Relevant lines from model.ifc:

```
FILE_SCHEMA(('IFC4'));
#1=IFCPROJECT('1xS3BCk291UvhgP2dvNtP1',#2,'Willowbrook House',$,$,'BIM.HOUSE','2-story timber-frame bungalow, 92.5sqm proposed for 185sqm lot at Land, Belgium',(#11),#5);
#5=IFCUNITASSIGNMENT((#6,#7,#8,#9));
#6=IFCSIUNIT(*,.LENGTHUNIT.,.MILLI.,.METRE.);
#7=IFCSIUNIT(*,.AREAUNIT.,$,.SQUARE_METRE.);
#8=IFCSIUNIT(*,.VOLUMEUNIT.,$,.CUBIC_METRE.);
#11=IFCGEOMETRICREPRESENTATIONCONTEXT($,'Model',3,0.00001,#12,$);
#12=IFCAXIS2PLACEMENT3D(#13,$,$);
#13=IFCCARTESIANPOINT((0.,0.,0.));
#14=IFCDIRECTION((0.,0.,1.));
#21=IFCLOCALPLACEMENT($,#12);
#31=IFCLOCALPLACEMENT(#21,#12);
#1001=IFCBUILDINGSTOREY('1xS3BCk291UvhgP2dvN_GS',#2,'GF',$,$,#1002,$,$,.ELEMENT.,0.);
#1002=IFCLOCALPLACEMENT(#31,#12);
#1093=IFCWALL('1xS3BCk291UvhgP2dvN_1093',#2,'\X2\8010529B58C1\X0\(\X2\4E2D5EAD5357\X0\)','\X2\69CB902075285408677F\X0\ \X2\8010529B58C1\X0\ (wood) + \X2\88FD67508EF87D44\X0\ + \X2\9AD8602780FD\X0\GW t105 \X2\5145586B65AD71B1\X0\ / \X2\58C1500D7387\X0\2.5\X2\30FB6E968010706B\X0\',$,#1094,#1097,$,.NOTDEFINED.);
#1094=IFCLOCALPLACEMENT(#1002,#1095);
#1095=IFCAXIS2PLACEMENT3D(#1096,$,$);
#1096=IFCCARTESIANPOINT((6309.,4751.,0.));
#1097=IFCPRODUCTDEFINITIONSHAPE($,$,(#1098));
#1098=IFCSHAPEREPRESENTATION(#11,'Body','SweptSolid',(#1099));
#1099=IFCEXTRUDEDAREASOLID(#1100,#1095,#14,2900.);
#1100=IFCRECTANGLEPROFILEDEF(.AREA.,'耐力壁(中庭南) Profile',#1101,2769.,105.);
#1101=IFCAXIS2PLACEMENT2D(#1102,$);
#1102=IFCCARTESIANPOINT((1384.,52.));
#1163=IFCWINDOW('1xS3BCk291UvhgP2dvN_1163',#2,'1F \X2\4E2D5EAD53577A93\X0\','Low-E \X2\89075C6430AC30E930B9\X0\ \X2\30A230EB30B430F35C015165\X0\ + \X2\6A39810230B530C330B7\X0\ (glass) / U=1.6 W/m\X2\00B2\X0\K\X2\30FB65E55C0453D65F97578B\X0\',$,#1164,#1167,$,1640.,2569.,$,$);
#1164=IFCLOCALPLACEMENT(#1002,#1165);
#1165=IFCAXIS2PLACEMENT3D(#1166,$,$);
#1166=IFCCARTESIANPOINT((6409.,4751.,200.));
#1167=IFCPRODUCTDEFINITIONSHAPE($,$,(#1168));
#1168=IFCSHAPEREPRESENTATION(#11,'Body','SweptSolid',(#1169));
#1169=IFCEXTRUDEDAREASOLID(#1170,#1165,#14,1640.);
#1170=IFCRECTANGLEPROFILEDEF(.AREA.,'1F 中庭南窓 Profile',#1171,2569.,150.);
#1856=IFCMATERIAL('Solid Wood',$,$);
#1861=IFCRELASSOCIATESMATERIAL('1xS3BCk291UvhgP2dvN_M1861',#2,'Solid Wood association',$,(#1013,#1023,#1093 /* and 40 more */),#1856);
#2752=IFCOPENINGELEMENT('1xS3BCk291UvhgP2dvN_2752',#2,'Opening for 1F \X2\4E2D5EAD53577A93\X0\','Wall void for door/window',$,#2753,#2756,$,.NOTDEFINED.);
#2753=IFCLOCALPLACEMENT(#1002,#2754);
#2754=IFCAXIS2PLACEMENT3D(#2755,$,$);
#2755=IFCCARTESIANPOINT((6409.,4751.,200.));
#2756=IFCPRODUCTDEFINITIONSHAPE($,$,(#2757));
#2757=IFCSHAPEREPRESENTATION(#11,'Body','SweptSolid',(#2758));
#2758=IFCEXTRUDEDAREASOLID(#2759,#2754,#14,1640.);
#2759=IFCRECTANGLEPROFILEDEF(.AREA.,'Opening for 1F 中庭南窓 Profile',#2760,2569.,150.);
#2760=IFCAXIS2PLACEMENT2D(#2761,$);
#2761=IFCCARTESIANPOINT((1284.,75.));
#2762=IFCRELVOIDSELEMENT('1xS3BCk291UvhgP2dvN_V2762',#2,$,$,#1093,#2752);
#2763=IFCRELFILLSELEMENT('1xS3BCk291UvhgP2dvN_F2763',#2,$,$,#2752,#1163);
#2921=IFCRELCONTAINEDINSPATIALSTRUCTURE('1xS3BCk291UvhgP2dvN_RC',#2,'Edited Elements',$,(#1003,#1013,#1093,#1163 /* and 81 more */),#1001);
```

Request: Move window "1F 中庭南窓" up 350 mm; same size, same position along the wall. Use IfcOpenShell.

```python
import numpy as np
import ifcopenshell
import ifcopenshell.api.geometry
import ifcopenshell.util.placement
import ifcopenshell.util.unit

model = ifcopenshell.open("model.ifc")
unit_scale = ifcopenshell.util.unit.calculate_unit_scale(model)

window = model.by_id(1163)
opening = window.FillsVoids[0].RelatingOpeningElement
dz = 350.0

shift = np.array([0.0, 0.0, dz])
# The window is not placed relative to its opening, so move both.
for product in (opening, window):
    matrix = ifcopenshell.util.placement.get_local_placement(product.ObjectPlacement)
    matrix[:3, 3] += shift
    ifcopenshell.api.geometry.edit_object_placement(model, product=product, matrix=matrix, is_si=False)

print(f"moved by {dz * unit_scale:+.3f} m")

model.write("model_v2.ifc")
```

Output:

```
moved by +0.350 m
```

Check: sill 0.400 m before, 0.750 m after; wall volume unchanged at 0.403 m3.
